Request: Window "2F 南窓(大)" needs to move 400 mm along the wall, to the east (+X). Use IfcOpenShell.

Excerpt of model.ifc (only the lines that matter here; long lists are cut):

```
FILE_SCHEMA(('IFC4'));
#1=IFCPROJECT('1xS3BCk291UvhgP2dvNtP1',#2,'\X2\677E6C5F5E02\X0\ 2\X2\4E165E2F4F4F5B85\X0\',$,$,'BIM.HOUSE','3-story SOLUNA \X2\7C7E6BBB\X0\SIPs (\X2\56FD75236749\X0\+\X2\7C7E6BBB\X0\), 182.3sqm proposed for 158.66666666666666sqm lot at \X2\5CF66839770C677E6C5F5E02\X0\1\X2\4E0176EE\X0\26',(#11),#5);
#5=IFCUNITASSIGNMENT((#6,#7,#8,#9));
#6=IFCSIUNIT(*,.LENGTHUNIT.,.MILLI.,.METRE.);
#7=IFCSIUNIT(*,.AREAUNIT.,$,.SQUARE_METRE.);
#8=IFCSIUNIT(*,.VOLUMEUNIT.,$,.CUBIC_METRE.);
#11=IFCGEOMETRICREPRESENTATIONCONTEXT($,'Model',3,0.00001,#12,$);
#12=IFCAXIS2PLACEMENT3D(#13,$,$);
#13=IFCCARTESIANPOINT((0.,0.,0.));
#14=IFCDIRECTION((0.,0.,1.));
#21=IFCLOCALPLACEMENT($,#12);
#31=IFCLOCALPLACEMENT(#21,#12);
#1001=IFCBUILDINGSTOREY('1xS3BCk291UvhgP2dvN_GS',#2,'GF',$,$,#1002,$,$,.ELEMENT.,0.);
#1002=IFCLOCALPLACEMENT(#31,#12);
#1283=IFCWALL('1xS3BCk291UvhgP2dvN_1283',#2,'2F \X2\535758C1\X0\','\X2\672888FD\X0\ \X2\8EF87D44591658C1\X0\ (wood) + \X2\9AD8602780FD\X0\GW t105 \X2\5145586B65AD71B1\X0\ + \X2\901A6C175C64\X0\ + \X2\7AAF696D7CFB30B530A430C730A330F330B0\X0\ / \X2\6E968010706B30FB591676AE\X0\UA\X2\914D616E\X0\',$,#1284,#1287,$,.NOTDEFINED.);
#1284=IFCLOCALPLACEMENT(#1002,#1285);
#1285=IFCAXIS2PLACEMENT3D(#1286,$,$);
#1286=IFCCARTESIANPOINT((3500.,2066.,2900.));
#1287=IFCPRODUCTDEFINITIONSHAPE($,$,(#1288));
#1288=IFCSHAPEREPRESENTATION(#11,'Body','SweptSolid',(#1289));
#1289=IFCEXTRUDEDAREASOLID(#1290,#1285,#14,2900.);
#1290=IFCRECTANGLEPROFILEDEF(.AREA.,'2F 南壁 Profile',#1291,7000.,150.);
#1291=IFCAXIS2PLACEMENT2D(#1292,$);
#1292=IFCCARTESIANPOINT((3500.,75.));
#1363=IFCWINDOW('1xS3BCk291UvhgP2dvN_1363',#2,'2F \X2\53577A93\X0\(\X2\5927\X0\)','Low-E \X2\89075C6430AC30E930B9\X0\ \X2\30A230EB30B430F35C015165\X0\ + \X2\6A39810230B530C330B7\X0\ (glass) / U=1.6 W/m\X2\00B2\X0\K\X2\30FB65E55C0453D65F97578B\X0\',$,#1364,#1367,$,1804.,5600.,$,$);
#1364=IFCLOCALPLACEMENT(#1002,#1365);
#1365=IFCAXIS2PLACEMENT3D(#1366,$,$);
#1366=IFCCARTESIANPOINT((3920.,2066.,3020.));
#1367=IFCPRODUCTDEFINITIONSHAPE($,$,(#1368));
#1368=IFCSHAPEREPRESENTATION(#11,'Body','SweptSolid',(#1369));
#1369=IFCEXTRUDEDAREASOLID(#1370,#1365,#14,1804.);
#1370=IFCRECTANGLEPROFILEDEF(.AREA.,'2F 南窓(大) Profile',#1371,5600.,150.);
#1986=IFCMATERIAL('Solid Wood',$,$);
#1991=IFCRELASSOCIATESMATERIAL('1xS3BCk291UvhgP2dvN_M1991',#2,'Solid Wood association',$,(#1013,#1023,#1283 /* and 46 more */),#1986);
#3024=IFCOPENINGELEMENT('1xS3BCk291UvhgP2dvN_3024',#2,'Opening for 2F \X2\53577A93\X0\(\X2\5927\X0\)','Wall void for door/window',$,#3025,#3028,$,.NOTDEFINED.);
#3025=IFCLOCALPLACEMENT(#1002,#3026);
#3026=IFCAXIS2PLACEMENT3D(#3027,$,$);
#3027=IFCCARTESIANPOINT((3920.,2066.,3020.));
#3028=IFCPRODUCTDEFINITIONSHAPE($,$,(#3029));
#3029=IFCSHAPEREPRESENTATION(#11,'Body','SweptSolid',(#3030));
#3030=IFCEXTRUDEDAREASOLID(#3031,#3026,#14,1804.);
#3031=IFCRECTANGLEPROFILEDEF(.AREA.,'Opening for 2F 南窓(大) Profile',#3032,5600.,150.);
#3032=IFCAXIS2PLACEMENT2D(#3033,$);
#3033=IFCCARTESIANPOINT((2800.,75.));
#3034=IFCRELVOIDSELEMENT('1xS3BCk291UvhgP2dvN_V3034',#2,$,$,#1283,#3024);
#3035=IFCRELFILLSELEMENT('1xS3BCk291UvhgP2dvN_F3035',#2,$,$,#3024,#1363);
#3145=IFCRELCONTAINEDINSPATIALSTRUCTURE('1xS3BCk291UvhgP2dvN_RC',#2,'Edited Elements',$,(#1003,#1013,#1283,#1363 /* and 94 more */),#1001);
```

```python
import ifcopenshell
import ifcopenshell.api.geometry
import ifcopenshell.util.placement
import ifcopenshell.util.unit

model = ifcopenshell.open("model.ifc")
unit_scale = ifcopenshell.util.unit.calculate_unit_scale(model)

window = model.by_id(1363)
opening = window.FillsVoids[0].RelatingOpeningElement
wall = opening.VoidsElements[0].RelatingBuildingElement

wall_matrix = ifcopenshell.util.placement.get_local_placement(wall.ObjectPlacement)
shift = wall_matrix[:3, 0] * 0.4 / unit_scale
before = ifcopenshell.util.placement.get_local_placement(window.ObjectPlacement)[:3, 3].copy()

# The window is not placed relative to its opening, so move both.
for product in (opening, window):
    matrix = ifcopenshell.util.placement.get_local_placement(product.ObjectPlacement)
    matrix[:3, 3] += shift
    ifcopenshell.api.geometry.edit_object_placement(model, product=product, matrix=matrix, is_si=False)

after = ifcopenshell.util.placement.get_local_placement(window.ObjectPlacement)[:3, 3]
print("window moved by", (after - before).round(3) + 0.0)

model.write("model_edited.ifc")
```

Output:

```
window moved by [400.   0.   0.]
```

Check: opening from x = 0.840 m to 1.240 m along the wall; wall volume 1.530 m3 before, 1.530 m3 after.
